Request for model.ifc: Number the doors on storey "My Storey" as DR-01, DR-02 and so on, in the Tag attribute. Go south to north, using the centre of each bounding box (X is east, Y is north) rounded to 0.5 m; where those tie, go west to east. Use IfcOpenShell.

First a look at what the model holds.

```python
import ifcopenshell
import ifcopenshell.util.element
import ifcopenshell.util.placement

model = ifcopenshell.open("model.ifc")
print(model.schema)
storey = next(s for s in model.by_type("IfcBuildingStorey") if s.Name == "My Storey")
doors = [e for e in ifcopenshell.util.element.get_decomposition(storey) if e.is_a("IfcDoor")]
for e in sorted(doors, key=lambda e: e.id()):
    origin = ifcopenshell.util.placement.get_local_placement(e.ObjectPlacement)[:3, 3]
    print(e.id(), e.Tag, e.Name, origin.round(2) + 0.0, sep=" | ")
```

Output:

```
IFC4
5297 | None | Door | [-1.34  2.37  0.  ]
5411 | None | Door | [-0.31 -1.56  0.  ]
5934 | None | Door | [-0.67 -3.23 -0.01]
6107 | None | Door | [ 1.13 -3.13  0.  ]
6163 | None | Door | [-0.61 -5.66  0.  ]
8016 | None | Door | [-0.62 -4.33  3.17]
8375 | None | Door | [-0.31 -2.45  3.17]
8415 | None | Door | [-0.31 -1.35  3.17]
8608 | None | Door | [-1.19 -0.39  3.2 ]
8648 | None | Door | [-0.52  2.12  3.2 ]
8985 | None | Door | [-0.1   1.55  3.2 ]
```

```python
import ifcopenshell
import ifcopenshell.geom
import ifcopenshell.util.element
import ifcopenshell.util.shape

model = ifcopenshell.open("model.ifc")
settings = ifcopenshell.geom.settings()
settings.set("use-world-coords", True)


def centre(element):
    shape = ifcopenshell.geom.create_shape(settings, element)
    return ifcopenshell.util.shape.get_bbox_centroid(shape.geometry)


storey = next(s for s in model.by_type("IfcBuildingStorey") if s.Name == "My Storey")
doors = [e for e in ifcopenshell.util.element.get_decomposition(storey) if e.is_a("IfcDoor")]

# Insertion points can sit at a corner or the storey origin, so sort by the geometry (in metres).
centres = {e: centre(e) for e in doors}
doors.sort(key=lambda e: (round(centres[e][1] / 0.5), centres[e][0]))

for i, e in enumerate(doors, start=1):
    number = f"DR-{i:02d}"
    e.Tag = number
    print(e.id(), number)

model.write("model_rev.ifc")
```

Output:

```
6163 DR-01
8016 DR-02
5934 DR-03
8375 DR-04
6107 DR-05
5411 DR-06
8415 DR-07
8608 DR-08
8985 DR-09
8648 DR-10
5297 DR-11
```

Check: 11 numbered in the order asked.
